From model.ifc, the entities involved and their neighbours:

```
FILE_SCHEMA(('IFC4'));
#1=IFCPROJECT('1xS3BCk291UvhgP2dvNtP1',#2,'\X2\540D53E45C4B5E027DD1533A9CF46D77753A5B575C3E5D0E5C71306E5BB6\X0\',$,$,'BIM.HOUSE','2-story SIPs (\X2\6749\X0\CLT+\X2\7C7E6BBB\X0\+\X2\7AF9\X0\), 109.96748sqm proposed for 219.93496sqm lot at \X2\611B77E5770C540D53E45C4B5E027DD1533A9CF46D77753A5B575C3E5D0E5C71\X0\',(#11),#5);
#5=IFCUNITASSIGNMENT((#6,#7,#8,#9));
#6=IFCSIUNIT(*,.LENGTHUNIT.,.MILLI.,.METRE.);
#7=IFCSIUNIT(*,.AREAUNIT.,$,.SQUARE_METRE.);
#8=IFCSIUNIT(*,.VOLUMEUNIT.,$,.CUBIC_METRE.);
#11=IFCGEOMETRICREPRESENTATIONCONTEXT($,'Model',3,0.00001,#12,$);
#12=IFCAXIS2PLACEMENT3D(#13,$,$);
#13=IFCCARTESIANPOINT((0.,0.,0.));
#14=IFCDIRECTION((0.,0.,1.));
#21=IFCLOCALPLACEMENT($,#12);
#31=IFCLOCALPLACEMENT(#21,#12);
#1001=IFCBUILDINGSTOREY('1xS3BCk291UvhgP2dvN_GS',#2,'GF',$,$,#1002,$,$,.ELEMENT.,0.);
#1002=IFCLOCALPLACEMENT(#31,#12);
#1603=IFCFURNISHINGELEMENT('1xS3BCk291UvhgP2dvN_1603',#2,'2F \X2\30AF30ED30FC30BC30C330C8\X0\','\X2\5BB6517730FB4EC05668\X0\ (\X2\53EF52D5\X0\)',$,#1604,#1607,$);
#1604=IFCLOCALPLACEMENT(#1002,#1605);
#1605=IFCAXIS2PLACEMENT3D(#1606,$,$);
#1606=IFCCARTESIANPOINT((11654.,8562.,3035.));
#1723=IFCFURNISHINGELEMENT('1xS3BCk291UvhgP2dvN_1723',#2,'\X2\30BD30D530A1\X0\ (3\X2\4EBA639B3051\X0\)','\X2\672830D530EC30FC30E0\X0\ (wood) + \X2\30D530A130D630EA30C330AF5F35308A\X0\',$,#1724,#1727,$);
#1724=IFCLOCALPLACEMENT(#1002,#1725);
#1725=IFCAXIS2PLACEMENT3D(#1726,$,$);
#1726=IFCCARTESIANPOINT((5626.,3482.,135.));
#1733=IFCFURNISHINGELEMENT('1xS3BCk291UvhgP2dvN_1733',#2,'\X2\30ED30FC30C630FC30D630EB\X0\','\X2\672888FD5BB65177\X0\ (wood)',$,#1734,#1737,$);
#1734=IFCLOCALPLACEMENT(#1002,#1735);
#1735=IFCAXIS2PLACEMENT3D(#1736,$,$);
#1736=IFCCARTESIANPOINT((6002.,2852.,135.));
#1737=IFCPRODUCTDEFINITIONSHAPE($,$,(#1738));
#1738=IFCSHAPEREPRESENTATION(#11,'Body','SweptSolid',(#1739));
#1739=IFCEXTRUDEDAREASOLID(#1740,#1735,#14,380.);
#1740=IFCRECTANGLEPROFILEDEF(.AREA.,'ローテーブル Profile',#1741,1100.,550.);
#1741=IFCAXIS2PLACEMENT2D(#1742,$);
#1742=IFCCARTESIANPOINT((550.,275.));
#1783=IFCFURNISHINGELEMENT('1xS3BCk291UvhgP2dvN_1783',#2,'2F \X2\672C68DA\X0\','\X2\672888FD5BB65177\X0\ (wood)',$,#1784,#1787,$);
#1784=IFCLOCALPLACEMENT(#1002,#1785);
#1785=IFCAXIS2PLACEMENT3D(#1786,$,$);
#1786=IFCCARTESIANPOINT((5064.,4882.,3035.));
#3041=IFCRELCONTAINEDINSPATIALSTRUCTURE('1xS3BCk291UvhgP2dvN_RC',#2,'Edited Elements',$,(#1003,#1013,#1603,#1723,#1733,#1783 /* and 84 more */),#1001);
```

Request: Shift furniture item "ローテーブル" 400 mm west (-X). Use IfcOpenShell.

```python
import ifcopenshell
import ifcopenshell.api.geometry
import ifcopenshell.util.placement
import ifcopenshell.util.unit

model = ifcopenshell.open("model.ifc")
unit_scale = ifcopenshell.util.unit.calculate_unit_scale(model)

item = model.by_guid("1xS3BCk291UvhgP2dvN_1733")
matrix = ifcopenshell.util.placement.get_local_placement(item.ObjectPlacement)
matrix[0, 3] -= 0.4 / unit_scale
ifcopenshell.api.geometry.edit_object_placement(model, product=item, matrix=matrix, is_si=False)

print(ifcopenshell.util.placement.get_local_placement(item.ObjectPlacement).round(3) + 0.0)

model.write("model_updated.ifc")
```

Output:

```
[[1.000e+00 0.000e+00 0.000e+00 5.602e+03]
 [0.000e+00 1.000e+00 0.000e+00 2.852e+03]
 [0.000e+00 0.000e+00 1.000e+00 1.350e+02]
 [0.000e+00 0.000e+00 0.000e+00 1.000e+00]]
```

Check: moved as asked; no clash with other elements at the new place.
